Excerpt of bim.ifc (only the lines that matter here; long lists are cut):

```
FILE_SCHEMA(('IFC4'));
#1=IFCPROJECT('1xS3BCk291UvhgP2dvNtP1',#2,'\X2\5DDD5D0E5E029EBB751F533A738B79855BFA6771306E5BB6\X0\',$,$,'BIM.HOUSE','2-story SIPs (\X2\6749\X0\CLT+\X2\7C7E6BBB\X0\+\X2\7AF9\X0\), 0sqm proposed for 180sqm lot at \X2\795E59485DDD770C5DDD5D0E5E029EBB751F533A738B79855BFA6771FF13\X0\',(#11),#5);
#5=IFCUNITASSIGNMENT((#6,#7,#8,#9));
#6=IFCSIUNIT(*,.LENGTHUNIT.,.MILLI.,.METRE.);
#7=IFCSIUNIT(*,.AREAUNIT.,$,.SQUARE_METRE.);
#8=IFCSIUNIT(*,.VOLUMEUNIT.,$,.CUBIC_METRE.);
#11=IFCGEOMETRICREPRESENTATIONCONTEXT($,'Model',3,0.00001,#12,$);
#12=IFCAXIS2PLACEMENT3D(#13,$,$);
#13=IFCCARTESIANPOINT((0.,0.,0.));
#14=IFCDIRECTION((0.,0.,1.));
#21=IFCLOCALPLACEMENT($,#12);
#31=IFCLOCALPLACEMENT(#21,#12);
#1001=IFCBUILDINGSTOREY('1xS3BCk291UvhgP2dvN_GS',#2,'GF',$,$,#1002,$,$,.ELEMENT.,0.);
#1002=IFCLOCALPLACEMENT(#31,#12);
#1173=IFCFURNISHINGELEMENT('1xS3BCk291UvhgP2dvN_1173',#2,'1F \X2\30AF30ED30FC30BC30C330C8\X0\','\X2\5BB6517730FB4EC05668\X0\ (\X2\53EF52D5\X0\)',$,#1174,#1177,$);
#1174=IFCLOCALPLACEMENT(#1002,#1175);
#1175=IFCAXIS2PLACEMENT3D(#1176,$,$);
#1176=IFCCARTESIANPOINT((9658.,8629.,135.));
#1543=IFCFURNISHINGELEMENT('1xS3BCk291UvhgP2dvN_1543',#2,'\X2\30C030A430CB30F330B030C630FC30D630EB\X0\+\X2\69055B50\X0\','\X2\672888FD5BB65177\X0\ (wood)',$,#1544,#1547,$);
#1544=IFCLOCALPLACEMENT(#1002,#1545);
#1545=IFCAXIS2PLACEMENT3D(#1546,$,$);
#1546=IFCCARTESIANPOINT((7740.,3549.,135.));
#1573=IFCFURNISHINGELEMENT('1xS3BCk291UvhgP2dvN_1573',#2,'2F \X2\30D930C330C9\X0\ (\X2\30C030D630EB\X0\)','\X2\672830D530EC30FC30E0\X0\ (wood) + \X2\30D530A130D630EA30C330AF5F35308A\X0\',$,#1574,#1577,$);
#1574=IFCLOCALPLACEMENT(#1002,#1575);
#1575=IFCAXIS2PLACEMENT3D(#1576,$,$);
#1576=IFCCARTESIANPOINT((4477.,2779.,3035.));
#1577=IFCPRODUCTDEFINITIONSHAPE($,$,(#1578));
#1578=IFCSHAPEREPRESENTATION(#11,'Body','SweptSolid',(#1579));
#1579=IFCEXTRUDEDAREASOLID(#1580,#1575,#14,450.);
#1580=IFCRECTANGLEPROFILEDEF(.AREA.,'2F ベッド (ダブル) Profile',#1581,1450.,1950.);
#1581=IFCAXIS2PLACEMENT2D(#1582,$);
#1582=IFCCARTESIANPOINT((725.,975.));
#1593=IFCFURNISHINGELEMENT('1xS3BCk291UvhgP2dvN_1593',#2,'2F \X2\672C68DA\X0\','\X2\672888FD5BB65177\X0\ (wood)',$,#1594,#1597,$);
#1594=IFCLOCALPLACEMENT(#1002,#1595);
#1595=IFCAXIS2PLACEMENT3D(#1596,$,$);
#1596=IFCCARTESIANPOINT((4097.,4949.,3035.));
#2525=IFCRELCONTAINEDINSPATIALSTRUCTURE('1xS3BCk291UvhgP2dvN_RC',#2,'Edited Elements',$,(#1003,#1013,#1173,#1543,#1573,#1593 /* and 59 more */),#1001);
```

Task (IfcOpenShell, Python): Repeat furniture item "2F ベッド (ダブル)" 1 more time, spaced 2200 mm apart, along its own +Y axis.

```python
import ifcopenshell
import ifcopenshell.api.geometry
import ifcopenshell.api.root
import ifcopenshell.util.element
import ifcopenshell.util.placement

model = ifcopenshell.open("bim.ifc")


def reuse_history(source, copy):
    """copy_class also copies each property set's owner history, people and application; keep the originals."""
    for rel in copy.IsDefinedBy:
        if rel.is_a("IfcRelDefinesByProperties") and (history := rel.RelatingPropertyDefinition.OwnerHistory):
            rel.RelatingPropertyDefinition.OwnerHistory = source.OwnerHistory
            ifcopenshell.util.element.remove_deep2(model, history)


source = model.by_guid("1xS3BCk291UvhgP2dvN_1573")
base = ifcopenshell.util.placement.get_local_placement(source.ObjectPlacement)
step = base[:3, 1] * 2200.0

for i in range(1, 2):
    copy = ifcopenshell.api.root.copy_class(model, product=source)
    copy.Representation = ifcopenshell.util.element.copy_deep(
        model, source.Representation, exclude=["IfcGeometricRepresentationContext", "IfcRepresentationMap"]
    )
    reuse_history(source, copy)
    matrix = base.copy()
    matrix[:3, 3] += i * step
    print("added at", matrix[:3, 3].round(3) + 0.0)
    ifcopenshell.api.geometry.edit_object_placement(model, product=copy, matrix=matrix, is_si=False)

model.write("bim_updated.ifc")
```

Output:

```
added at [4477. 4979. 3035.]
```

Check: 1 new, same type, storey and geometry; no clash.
